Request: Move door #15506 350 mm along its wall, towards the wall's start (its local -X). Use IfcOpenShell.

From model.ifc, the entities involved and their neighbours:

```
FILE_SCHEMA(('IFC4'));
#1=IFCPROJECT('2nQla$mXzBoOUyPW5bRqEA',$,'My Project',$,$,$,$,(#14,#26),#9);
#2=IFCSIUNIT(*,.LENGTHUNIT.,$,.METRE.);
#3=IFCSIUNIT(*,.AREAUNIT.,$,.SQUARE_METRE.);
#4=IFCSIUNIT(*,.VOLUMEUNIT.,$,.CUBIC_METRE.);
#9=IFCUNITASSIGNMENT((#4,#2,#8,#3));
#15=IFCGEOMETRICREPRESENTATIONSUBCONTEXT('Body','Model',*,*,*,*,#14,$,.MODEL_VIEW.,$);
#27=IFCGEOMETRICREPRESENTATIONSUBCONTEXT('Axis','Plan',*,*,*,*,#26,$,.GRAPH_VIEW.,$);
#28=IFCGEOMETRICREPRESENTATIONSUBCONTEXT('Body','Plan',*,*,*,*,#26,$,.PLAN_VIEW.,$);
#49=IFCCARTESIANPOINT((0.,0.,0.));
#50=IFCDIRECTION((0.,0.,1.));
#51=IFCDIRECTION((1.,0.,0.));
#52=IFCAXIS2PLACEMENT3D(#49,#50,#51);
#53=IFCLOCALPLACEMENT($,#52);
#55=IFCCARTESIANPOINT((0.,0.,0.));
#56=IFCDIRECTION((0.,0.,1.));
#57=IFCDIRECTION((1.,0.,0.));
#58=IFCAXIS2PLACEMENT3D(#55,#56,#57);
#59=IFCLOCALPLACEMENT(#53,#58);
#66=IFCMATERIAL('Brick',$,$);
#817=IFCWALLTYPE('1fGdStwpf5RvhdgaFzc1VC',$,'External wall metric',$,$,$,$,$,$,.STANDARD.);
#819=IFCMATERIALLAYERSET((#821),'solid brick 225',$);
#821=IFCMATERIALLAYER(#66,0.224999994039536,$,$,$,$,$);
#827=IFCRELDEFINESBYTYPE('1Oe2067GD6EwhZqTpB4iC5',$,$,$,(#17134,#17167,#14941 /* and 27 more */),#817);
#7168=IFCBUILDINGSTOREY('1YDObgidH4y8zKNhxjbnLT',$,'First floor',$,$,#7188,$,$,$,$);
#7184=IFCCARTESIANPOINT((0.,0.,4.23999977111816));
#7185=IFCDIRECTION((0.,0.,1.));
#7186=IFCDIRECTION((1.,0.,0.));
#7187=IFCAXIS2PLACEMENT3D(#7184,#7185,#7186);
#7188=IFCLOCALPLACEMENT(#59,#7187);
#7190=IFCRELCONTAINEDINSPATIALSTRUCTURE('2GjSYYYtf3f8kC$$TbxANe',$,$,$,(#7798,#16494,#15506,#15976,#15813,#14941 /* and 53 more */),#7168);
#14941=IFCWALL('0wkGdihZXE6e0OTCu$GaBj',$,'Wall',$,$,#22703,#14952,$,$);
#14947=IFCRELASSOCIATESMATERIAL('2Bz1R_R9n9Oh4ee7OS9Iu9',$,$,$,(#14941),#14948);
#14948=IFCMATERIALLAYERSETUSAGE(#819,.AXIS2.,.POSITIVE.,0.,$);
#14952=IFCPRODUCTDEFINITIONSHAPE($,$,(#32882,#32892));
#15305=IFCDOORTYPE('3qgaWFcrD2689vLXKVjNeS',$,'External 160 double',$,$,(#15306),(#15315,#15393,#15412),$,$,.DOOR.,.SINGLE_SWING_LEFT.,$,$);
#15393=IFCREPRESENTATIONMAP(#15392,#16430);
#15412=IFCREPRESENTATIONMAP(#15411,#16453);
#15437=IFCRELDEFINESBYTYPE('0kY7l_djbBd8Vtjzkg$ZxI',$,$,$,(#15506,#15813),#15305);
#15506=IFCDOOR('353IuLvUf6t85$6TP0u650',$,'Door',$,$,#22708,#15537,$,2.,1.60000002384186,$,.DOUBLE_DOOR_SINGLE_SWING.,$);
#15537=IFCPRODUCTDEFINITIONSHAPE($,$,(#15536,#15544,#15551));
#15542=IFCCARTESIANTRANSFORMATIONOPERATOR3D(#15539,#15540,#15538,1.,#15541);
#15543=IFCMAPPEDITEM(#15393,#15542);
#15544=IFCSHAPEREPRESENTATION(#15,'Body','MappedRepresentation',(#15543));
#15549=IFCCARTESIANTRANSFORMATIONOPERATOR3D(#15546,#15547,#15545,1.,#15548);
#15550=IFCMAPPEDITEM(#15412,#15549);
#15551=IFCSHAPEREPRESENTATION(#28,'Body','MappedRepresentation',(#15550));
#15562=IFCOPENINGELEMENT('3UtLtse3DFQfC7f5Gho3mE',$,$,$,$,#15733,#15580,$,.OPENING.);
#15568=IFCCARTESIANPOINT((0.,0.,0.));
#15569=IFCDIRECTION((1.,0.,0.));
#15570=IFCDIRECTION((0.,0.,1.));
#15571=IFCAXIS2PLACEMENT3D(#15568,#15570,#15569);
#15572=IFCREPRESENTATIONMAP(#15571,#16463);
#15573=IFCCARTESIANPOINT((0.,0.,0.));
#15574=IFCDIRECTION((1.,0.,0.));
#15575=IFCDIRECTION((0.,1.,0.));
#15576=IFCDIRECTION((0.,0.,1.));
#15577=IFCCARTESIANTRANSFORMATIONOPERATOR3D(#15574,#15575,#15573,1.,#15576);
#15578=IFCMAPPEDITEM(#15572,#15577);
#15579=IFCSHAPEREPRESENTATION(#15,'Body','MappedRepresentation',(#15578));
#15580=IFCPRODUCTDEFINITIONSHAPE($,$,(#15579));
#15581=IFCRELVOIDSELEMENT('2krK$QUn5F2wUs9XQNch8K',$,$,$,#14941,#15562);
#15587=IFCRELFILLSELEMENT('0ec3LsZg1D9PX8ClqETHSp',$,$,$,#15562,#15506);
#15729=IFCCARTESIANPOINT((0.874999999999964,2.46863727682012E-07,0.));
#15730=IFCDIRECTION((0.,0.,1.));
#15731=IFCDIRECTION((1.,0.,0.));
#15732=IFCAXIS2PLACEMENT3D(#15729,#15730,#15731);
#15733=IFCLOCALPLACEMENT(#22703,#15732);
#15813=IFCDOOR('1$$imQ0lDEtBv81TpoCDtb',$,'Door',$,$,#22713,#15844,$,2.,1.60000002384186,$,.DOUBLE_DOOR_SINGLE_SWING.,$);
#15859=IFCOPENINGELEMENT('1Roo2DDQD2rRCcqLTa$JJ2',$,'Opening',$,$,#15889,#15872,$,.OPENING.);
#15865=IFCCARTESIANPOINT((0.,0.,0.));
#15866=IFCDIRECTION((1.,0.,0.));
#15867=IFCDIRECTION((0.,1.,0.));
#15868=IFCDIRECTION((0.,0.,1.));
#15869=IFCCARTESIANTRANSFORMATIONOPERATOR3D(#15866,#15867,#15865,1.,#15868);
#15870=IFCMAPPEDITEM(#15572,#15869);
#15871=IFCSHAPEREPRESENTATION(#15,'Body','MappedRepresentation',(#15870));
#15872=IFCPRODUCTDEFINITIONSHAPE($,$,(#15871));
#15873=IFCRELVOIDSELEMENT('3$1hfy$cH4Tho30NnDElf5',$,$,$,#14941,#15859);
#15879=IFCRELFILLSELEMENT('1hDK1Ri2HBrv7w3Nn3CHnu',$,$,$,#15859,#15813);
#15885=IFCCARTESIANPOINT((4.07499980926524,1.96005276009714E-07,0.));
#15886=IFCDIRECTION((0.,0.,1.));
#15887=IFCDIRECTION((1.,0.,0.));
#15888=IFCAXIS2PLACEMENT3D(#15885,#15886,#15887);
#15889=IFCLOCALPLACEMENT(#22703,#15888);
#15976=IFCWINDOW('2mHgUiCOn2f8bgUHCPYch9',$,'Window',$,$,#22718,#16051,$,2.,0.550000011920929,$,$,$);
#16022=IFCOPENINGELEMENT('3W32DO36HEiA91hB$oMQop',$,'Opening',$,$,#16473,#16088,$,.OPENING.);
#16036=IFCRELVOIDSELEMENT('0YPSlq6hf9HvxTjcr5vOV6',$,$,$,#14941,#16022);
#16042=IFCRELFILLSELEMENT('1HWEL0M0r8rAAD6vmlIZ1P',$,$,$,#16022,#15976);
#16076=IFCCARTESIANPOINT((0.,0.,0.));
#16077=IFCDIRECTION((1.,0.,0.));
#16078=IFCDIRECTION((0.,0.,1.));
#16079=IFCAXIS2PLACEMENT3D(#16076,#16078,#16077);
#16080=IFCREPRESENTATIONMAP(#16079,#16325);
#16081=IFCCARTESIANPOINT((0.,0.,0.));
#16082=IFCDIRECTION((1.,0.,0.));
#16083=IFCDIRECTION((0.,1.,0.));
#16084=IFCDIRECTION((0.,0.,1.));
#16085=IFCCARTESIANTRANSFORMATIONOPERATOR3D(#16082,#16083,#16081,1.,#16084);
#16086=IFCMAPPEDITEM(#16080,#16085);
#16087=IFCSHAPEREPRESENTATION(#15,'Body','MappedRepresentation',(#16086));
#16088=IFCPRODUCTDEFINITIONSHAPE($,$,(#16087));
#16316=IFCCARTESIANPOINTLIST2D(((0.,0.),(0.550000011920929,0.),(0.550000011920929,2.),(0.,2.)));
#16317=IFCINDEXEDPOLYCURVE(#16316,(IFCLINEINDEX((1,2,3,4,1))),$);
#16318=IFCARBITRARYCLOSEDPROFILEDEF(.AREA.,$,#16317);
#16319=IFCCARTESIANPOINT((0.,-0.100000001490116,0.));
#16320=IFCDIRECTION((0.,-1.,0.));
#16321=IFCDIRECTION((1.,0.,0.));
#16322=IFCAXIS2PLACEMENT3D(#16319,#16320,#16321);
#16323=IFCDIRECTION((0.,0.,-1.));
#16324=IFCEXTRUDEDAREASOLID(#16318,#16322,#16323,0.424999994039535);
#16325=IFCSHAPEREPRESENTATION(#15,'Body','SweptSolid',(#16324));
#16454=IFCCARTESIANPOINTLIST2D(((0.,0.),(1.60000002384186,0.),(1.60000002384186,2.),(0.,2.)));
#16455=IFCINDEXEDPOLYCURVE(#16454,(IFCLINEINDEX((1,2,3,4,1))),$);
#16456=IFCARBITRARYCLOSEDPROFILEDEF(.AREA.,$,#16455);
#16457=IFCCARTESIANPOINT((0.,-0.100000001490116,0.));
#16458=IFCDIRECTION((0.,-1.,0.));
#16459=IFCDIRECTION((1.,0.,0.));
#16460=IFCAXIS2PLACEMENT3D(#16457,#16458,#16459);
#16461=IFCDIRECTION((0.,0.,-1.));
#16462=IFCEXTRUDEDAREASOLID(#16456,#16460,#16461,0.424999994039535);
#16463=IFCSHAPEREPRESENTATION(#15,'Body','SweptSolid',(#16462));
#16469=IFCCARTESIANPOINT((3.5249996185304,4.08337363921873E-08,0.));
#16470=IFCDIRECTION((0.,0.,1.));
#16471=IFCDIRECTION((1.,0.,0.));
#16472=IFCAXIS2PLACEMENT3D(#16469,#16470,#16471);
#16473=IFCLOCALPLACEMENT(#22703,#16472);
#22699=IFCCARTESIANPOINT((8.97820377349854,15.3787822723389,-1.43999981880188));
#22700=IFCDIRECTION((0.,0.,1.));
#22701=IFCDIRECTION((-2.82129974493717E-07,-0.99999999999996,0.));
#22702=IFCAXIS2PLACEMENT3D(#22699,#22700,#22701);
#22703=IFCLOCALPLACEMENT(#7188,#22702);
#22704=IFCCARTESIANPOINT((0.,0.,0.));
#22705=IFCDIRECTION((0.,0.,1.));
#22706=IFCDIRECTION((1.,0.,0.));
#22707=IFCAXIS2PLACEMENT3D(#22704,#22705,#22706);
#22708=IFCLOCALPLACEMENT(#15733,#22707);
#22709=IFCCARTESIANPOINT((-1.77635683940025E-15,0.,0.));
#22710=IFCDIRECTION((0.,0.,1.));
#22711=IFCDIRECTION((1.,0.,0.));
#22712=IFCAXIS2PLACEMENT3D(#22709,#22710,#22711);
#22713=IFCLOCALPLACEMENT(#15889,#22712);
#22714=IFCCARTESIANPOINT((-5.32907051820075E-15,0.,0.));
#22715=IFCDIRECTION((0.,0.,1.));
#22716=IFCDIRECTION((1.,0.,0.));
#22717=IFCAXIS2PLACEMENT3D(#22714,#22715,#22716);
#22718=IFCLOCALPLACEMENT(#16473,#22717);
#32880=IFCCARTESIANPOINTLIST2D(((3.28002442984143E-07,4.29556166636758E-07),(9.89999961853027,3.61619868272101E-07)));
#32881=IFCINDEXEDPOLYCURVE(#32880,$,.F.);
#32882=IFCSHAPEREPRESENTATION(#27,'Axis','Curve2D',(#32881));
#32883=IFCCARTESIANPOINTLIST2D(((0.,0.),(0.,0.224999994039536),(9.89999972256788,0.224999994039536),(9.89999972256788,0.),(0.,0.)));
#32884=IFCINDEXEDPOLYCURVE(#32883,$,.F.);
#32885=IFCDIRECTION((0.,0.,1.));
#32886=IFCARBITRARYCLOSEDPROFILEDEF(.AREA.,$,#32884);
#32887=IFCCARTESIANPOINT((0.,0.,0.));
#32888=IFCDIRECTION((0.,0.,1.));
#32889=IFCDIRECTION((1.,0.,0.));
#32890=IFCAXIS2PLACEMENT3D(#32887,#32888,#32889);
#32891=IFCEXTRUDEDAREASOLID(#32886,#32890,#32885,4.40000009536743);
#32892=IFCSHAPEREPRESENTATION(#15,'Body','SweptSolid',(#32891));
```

```python
import ifcopenshell
import ifcopenshell.api.geometry
import ifcopenshell.util.placement
import ifcopenshell.util.unit

model = ifcopenshell.open("model.ifc")
unit_scale = ifcopenshell.util.unit.calculate_unit_scale(model)

door = model.by_guid("353IuLvUf6t85$6TP0u650")
opening = door.FillsVoids[0].RelatingOpeningElement
wall = opening.VoidsElements[0].RelatingBuildingElement

wall_matrix = ifcopenshell.util.placement.get_local_placement(wall.ObjectPlacement)
shift = wall_matrix[:3, 0] * -0.35 / unit_scale
before = ifcopenshell.util.placement.get_local_placement(door.ObjectPlacement)[:3, 3].copy()

# The door is placed relative to its opening, so it follows when the opening moves.
matrix = ifcopenshell.util.placement.get_local_placement(opening.ObjectPlacement)
matrix[:3, 3] += shift
ifcopenshell.api.geometry.edit_object_placement(
    model, product=opening, matrix=matrix, is_si=False, should_transform_children=True
)

after = ifcopenshell.util.placement.get_local_placement(door.ObjectPlacement)[:3, 3]
print("door moved by", (after - before).round(3) + 0.0)

model.write("model_updated.ifc")
```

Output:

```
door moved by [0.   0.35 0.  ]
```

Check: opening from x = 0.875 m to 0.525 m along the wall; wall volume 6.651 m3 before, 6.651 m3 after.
